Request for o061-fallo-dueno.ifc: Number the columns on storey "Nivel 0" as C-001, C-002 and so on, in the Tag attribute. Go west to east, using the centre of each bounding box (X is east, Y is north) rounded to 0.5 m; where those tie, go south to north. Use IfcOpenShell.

First a look at what the model holds.

```python
import ifcopenshell
import ifcopenshell.util.element
import ifcopenshell.util.placement

model = ifcopenshell.open("o061-fallo-dueno.ifc")
print(model.schema)
storey = next(s for s in model.by_type("IfcBuildingStorey") if s.Name == "Nivel 0")
columns = [e for e in ifcopenshell.util.element.get_decomposition(storey) if e.is_a("IfcColumn")]
for e in sorted(columns, key=lambda e: e.id()):
    origin = ifcopenshell.util.placement.get_local_placement(e.ObjectPlacement)[:3, 3]
    print(e.id(), e.Tag, e.Name, origin.round(2) + 0.0, sep=" | ")
```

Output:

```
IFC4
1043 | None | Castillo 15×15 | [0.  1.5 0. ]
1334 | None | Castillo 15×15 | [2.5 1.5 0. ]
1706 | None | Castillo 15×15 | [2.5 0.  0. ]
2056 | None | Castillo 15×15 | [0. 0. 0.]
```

```python
import ifcopenshell
import ifcopenshell.geom
import ifcopenshell.util.element
import ifcopenshell.util.shape

model = ifcopenshell.open("o061-fallo-dueno.ifc")
settings = ifcopenshell.geom.settings()
settings.set("use-world-coords", True)


def centre(element):
    shape = ifcopenshell.geom.create_shape(settings, element)
    return ifcopenshell.util.shape.get_bbox_centroid(shape.geometry)


storey = next(s for s in model.by_type("IfcBuildingStorey") if s.Name == "Nivel 0")
columns = [e for e in ifcopenshell.util.element.get_decomposition(storey) if e.is_a("IfcColumn")]

# Insertion points can sit at a corner or the storey origin, so sort by the geometry (in metres).
centres = {e: centre(e) for e in columns}
columns.sort(key=lambda e: (round(centres[e][0] / 0.5), centres[e][1]))

for i, e in enumerate(columns, start=1):
    number = f"C-0{i:02d}"
    e.Tag = number
    print(e.id(), number)

model.write("o061-fallo-dueno_v2.ifc")
```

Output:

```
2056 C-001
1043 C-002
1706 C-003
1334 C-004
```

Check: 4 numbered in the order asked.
